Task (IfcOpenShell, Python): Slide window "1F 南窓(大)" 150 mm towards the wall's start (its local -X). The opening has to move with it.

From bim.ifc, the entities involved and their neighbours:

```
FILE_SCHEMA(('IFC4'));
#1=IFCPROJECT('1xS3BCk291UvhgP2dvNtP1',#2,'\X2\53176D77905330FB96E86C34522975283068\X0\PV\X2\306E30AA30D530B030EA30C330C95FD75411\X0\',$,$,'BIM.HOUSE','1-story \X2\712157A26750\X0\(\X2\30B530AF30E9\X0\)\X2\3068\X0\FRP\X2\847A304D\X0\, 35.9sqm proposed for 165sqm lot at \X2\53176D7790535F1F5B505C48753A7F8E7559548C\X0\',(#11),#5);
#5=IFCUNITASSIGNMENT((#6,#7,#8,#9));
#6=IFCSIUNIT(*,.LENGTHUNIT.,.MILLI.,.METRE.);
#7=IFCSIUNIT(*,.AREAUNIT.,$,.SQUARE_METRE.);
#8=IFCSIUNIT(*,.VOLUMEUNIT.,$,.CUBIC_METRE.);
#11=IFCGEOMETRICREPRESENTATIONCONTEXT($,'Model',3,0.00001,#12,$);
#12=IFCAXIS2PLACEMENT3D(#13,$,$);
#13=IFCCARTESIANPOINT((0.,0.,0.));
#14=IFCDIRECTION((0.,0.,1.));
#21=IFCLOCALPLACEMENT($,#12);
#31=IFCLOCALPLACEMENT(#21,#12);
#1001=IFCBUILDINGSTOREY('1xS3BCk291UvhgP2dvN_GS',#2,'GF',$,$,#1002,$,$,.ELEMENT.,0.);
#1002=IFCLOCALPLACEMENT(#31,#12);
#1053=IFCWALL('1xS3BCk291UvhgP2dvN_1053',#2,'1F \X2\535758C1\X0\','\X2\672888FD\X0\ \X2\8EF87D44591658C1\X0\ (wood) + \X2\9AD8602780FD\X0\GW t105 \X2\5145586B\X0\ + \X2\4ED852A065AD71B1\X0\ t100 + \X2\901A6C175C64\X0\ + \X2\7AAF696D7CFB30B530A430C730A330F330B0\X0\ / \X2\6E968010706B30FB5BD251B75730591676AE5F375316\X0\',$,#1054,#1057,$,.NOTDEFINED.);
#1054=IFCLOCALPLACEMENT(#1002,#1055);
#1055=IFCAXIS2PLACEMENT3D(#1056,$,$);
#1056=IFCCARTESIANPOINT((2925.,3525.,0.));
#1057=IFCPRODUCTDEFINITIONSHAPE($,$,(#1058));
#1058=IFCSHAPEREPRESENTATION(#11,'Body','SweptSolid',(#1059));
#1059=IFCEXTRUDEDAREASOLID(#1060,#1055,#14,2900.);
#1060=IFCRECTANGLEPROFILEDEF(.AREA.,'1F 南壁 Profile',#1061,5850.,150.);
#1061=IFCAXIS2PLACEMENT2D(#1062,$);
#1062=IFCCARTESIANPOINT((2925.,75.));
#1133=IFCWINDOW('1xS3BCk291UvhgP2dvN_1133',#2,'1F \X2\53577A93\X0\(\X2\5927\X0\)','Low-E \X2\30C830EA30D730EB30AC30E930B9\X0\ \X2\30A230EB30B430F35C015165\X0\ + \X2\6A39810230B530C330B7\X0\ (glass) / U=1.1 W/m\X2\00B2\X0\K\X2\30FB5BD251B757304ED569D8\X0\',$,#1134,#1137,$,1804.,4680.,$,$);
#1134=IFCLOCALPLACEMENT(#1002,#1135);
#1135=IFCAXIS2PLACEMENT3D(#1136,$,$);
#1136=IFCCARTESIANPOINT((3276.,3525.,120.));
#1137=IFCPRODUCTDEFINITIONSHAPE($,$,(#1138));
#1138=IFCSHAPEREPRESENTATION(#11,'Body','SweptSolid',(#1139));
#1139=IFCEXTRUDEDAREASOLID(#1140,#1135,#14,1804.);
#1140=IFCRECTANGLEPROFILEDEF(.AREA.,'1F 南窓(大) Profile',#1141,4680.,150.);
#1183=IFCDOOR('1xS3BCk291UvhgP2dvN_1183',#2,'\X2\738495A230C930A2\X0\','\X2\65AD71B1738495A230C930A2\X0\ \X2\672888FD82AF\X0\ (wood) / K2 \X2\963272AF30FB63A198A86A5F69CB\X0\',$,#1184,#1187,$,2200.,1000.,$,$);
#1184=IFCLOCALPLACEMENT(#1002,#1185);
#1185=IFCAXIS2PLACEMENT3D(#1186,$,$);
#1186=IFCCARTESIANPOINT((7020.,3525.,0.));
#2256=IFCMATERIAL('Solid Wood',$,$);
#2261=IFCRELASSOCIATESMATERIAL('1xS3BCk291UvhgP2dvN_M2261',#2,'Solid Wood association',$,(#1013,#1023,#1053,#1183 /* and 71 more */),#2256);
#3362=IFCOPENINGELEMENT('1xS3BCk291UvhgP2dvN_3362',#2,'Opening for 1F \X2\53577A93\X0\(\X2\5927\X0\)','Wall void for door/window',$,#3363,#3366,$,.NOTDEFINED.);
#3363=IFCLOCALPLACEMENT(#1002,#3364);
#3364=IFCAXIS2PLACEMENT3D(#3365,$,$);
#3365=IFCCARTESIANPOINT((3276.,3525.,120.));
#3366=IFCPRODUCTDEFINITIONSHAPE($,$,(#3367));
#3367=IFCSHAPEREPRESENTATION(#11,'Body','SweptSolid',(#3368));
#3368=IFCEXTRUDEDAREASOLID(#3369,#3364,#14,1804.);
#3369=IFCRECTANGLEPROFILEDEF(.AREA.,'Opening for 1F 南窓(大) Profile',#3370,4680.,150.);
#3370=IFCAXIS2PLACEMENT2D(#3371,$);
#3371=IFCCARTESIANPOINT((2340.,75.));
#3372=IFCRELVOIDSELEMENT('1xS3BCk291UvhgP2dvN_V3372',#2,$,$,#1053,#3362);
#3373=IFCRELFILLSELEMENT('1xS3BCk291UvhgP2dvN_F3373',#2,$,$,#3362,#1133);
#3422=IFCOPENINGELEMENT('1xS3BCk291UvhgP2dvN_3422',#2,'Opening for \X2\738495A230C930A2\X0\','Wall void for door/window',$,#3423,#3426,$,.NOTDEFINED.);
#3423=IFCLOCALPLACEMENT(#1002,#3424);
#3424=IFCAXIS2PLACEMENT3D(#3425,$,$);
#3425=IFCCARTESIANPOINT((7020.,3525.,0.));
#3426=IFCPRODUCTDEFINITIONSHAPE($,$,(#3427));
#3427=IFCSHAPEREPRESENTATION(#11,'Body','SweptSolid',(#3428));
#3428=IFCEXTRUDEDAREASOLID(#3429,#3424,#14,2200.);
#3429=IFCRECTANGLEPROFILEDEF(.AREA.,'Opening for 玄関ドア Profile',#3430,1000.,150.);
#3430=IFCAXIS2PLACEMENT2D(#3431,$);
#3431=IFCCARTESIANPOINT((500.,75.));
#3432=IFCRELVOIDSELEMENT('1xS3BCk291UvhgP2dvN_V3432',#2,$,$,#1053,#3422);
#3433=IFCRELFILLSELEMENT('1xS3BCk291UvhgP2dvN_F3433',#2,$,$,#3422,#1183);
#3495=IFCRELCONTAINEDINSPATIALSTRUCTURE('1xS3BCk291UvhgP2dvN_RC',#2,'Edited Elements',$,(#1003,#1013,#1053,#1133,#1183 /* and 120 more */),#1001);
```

```python
import ifcopenshell
import ifcopenshell.api.geometry
import ifcopenshell.util.placement

model = ifcopenshell.open("bim.ifc")

window = model.by_guid("1xS3BCk291UvhgP2dvN_1133")
opening = window.FillsVoids[0].RelatingOpeningElement
wall = opening.VoidsElements[0].RelatingBuildingElement

wall_matrix = ifcopenshell.util.placement.get_local_placement(wall.ObjectPlacement)
shift = wall_matrix[:3, 0] * -150.0
before = ifcopenshell.util.placement.get_local_placement(window.ObjectPlacement)[:3, 3].copy()

# The window is not placed relative to its opening, so move both.
for product in (opening, window):
    matrix = ifcopenshell.util.placement.get_local_placement(product.ObjectPlacement)
    matrix[:3, 3] += shift
    ifcopenshell.api.geometry.edit_object_placement(model, product=product, matrix=matrix, is_si=False)

after = ifcopenshell.util.placement.get_local_placement(window.ObjectPlacement)[:3, 3]
print("window moved by", (after - before).round(3) + 0.0)

model.write("bim_edited.ifc")
```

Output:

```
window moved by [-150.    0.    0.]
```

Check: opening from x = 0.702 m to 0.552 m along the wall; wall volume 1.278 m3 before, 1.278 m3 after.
